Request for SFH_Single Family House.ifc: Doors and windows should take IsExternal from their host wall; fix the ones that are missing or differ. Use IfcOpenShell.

First a look at what the model holds.

```python
import ifcopenshell
import ifcopenshell.util.element

model = ifcopenshell.open("SFH_Single Family House.ifc")
print(model.schema)
seen = {}
for e in model.by_type("IfcDoor") + model.by_type("IfcWindow"):
    if not e.FillsVoids:
        continue
    host = e.FillsVoids[0].RelatingOpeningElement.VoidsElements[0].RelatingBuildingElement
    own = ifcopenshell.util.element.get_pset(e, f"Pset_{e.is_a()[3:].removesuffix('StandardCase')}Common", "IsExternal")
    wall = ifcopenshell.util.element.get_pset(host, "Pset_WallCommon", "IsExternal")
    seen[e.is_a(), own, wall] = seen.get((e.is_a(), own, wall), 0) + 1
for (cls, own, wall), count in sorted(seen.items(), key=str):
    print(count, cls, "IsExternal:", own, "| host wall:", wall)
```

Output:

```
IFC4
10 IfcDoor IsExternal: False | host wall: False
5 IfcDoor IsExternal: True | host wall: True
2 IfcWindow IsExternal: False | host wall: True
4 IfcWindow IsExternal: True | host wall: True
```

```python
import ifcopenshell
import ifcopenshell.api.pset
import ifcopenshell.util.element

model = ifcopenshell.open("SFH_Single Family House.ifc")

count = 0
for ifc_class, pset_name in (("IfcDoor", "Pset_DoorCommon"), ("IfcWindow", "Pset_WindowCommon")):
    for e in model.by_type(ifc_class):
        if not e.FillsVoids:
            continue
        host = e.FillsVoids[0].RelatingOpeningElement.VoidsElements[0].RelatingBuildingElement
        external = ifcopenshell.util.element.get_pset(host, "Pset_WallCommon", "IsExternal")
        if external is None or ifcopenshell.util.element.get_pset(e, pset_name, "IsExternal") == external:
            continue
        pset = ifcopenshell.api.pset.add_pset(model, product=e, name=pset_name)
        ifcopenshell.api.pset.edit_pset(model, pset=pset, properties={"IsExternal": external})
        count += 1

print(count, "updated")

model.write("SFH_Single Family House-out.ifc")
```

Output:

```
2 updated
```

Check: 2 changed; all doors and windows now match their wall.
